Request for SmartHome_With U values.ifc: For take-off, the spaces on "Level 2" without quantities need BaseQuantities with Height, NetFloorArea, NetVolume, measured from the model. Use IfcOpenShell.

First a look at what the model holds.

```python
import ifcopenshell
import ifcopenshell.util.element
import ifcopenshell.util.unit

model = ifcopenshell.open("SmartHome_With U values.ifc")
print(model.schema)
for unit_type in ("LENGTHUNIT", "AREAUNIT", "VOLUMEUNIT"):
    print(unit_type, ifcopenshell.util.unit.calculate_unit_scale(model, unit_type))
storey = next(s for s in model.by_type("IfcBuildingStorey") if s.Name == "Level 2")
spaces = [e for e in ifcopenshell.util.element.get_decomposition(storey) if e.is_a("IfcSpace")]
for e in sorted(spaces, key=lambda e: e.id()):
    print(e.id(), e.is_a(), e.Name, list(ifcopenshell.util.element.get_psets(e, qtos_only=True)), sep=" | ")
```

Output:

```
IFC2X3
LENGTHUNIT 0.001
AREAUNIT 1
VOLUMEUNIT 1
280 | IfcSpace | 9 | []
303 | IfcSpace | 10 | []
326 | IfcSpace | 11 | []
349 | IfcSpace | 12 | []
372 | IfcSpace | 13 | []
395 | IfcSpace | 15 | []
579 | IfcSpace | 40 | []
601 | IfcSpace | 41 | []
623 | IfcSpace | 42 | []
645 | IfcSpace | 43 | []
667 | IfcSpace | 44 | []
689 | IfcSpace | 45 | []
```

```python
import ifcopenshell
import ifcopenshell.api.pset
import ifcopenshell.geom
import ifcopenshell.util.element
import ifcopenshell.util.shape
import ifcopenshell.util.unit

model = ifcopenshell.open("SmartHome_With U values.ifc")
unit_scale = ifcopenshell.util.unit.calculate_unit_scale(model)
area_scale = ifcopenshell.util.unit.calculate_unit_scale(model, "AREAUNIT")
volume_scale = ifcopenshell.util.unit.calculate_unit_scale(model, "VOLUMEUNIT")
settings = ifcopenshell.geom.settings()

storey = next(s for s in model.by_type("IfcBuildingStorey") if s.Name == "Level 2")
spaces = [e for e in ifcopenshell.util.element.get_decomposition(storey) if e.is_a("IfcSpace")]

for e in sorted(spaces, key=lambda e: e.id()):
    if ifcopenshell.util.element.get_psets(e, qtos_only=True, should_inherit=False):
        continue
    # Geometry comes back in metres, in the element's own axes.
    shape = ifcopenshell.geom.create_shape(settings, e)
    values = {
        "Height": ifcopenshell.util.shape.get_z(shape.geometry) / unit_scale,
        "NetFloorArea": ifcopenshell.util.shape.get_footprint_area(shape.geometry) / area_scale,
        "NetVolume": ifcopenshell.util.shape.get_volume(shape.geometry) / volume_scale,
    }
    qto = ifcopenshell.api.pset.add_qto(model, product=e, name="BaseQuantities")
    ifcopenshell.api.pset.edit_qto(model, qto=qto, properties=values)
    print(e.id(), {k: round(v, 3) for k, v in values.items()})

model.write("SmartHome_With U values_rev.ifc")
```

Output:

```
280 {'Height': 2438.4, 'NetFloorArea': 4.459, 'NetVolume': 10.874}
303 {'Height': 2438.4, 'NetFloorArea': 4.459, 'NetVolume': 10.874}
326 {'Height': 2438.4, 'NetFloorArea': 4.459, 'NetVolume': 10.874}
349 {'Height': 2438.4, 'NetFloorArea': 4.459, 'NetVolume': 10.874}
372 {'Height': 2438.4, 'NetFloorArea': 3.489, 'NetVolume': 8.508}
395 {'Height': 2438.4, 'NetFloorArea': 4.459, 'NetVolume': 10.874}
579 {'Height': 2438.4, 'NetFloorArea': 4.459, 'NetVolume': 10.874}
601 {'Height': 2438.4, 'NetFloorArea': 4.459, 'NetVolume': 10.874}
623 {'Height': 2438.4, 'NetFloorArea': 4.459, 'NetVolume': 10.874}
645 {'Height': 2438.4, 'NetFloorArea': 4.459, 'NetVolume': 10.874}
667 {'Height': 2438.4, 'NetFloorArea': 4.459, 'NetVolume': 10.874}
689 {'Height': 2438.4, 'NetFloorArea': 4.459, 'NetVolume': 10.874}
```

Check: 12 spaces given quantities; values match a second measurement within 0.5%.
